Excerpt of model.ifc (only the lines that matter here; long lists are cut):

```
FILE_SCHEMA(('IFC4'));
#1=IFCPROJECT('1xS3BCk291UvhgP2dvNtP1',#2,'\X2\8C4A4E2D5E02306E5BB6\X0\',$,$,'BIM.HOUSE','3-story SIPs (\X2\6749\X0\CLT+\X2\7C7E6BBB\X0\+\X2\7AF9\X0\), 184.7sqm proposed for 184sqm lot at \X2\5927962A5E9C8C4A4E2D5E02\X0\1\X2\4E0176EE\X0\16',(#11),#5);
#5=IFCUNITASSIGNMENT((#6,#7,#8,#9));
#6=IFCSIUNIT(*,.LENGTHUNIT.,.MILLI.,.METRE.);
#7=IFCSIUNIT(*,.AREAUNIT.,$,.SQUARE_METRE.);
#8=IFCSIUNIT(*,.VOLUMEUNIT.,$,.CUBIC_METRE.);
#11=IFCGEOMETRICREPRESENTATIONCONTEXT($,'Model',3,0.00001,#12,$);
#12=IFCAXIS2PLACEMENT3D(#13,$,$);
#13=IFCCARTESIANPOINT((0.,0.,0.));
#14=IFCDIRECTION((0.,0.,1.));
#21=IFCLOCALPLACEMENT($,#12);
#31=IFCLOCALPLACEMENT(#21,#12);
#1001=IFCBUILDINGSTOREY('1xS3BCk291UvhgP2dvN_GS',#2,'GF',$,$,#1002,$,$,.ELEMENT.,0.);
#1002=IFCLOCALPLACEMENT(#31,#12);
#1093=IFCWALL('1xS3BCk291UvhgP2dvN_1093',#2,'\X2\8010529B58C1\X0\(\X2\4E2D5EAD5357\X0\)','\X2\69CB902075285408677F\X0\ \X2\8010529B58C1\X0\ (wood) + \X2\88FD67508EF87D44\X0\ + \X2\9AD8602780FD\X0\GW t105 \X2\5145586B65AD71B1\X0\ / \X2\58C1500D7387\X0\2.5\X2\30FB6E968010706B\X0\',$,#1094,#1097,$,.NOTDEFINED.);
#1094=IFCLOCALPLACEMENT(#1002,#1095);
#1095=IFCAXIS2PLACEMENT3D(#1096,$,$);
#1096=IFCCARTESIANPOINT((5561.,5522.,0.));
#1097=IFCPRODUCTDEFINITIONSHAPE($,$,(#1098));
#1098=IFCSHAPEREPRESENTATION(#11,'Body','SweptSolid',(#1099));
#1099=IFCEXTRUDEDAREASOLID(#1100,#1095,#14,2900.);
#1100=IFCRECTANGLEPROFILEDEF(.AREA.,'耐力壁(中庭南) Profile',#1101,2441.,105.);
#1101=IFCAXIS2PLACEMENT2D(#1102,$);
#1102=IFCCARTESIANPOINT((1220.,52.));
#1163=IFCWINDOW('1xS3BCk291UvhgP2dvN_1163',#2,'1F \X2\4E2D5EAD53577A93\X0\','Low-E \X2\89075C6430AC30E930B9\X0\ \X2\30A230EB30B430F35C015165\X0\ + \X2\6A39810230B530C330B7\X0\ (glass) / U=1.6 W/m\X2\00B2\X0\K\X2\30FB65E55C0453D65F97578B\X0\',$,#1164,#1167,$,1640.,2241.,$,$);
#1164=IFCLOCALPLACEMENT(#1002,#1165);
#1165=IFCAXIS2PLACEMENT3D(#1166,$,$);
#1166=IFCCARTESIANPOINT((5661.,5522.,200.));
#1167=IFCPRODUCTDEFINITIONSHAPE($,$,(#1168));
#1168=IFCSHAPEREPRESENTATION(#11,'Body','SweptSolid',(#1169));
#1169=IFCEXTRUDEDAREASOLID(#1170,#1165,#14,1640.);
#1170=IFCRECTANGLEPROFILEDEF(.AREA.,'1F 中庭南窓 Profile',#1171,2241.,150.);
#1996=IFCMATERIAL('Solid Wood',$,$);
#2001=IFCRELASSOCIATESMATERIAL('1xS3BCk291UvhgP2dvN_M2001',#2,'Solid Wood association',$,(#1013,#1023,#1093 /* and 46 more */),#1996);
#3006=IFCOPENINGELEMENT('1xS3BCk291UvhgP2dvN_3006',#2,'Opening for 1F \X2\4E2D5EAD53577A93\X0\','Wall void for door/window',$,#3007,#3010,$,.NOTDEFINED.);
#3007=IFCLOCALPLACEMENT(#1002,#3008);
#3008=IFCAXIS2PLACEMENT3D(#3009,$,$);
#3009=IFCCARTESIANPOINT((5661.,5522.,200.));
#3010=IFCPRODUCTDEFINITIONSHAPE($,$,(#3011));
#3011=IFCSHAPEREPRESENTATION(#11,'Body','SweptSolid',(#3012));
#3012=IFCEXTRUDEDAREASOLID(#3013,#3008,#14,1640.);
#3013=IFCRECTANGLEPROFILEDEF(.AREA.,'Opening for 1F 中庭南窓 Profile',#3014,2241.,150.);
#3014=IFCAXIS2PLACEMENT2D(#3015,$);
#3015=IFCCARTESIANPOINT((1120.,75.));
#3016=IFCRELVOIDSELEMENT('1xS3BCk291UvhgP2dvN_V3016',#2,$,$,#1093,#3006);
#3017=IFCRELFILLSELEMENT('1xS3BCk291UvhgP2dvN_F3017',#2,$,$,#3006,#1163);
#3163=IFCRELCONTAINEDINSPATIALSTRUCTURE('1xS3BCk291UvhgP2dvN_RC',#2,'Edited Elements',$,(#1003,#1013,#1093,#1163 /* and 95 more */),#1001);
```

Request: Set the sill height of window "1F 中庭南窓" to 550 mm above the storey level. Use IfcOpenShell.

```python
import numpy as np
import ifcopenshell
import ifcopenshell.api.geometry
import ifcopenshell.geom
import ifcopenshell.util.element
import ifcopenshell.util.placement
import ifcopenshell.util.shape
import ifcopenshell.util.unit

model = ifcopenshell.open("model.ifc")
unit_scale = ifcopenshell.util.unit.calculate_unit_scale(model)

window = model.by_guid("1xS3BCk291UvhgP2dvN_1163")
opening = window.FillsVoids[0].RelatingOpeningElement
storey = ifcopenshell.util.element.get_container(window, ifc_class="IfcBuildingStorey")
level = ifcopenshell.util.placement.get_local_placement(storey.ObjectPlacement)[2, 3]

# The opening's origin need not be at the sill, so measure its lowest point.
shape = ifcopenshell.geom.create_shape(ifcopenshell.geom.settings(), opening)
bottom = ifcopenshell.util.shape.get_shape_bottom_elevation(shape, shape.geometry) / unit_scale
dz = level + 0.55 / unit_scale - bottom

shift = np.array([0.0, 0.0, dz])
# The window is not placed relative to its opening, so move both.
for product in (opening, window):
    matrix = ifcopenshell.util.placement.get_local_placement(product.ObjectPlacement)
    matrix[:3, 3] += shift
    ifcopenshell.api.geometry.edit_object_placement(model, product=product, matrix=matrix, is_si=False)

print(f"moved by {dz * unit_scale:+.3f} m")

model.write("model_edited.ifc")
```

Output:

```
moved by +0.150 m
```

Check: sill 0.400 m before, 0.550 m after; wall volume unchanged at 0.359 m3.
